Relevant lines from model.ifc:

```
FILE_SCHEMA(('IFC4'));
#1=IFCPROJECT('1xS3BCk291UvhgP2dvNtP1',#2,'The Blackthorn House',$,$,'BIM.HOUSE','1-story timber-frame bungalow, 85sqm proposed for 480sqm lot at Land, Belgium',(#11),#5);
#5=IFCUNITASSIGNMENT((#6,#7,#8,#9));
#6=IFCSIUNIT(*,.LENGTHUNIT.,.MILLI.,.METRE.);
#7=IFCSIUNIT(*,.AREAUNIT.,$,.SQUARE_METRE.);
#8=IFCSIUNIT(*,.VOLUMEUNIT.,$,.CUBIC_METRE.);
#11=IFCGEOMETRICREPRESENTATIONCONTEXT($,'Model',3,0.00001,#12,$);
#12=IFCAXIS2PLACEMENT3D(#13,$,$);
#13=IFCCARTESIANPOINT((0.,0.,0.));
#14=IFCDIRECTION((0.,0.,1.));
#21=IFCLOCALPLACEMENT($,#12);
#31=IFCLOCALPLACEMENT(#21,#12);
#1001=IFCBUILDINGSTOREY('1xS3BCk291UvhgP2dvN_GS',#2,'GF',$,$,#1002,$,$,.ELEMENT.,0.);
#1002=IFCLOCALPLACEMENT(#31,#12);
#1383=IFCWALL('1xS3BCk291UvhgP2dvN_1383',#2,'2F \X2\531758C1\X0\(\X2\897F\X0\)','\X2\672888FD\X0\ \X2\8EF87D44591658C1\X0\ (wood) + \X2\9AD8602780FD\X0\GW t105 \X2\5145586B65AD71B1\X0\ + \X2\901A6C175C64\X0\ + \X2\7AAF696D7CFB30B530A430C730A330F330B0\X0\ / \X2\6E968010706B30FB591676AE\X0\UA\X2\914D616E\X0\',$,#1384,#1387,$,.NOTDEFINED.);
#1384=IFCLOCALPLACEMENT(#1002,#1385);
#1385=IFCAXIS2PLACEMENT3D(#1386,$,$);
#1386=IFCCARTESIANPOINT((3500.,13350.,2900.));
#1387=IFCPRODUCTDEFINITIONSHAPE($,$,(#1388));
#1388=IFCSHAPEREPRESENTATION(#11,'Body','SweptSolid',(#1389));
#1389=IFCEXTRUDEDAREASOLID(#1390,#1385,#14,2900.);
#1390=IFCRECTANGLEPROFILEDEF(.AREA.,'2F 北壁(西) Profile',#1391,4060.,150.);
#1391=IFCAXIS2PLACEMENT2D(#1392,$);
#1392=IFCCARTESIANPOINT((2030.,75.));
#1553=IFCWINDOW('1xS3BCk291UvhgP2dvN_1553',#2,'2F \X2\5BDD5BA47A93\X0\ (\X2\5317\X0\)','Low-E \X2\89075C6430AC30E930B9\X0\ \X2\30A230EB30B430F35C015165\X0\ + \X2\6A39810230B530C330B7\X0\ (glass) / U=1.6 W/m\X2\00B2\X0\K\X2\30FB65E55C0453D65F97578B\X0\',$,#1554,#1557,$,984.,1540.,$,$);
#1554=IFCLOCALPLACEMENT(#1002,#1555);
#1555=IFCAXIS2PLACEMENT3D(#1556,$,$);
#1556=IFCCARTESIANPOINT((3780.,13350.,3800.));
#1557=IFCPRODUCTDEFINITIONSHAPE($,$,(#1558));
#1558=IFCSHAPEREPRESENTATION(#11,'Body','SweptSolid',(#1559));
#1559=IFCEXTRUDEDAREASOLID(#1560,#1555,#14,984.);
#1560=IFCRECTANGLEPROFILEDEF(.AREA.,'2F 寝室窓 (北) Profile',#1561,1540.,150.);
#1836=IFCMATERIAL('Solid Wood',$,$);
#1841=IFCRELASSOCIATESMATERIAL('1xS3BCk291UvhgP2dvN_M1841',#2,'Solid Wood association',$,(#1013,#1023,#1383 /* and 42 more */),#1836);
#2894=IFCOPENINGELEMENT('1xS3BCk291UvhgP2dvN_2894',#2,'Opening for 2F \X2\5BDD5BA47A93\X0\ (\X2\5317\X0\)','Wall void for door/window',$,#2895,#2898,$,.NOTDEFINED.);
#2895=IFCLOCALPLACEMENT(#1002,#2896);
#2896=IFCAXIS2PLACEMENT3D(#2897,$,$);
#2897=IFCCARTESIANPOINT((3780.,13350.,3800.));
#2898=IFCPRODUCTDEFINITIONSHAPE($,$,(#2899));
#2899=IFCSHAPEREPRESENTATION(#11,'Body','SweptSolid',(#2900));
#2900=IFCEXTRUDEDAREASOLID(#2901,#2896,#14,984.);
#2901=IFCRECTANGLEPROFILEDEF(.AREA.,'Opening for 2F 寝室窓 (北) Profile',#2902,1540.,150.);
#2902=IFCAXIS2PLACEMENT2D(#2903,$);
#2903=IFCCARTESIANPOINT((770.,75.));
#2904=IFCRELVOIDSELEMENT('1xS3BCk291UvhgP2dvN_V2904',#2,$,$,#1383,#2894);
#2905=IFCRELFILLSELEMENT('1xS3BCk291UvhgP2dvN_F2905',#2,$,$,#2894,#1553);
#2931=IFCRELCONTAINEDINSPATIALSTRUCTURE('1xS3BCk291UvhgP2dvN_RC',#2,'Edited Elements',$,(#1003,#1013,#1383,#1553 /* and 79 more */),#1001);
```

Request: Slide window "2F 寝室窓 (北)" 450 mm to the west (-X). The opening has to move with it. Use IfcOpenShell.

```python
import ifcopenshell
import ifcopenshell.api.geometry
import ifcopenshell.util.placement

model = ifcopenshell.open("model.ifc")

window = model.by_id(1553)
opening = window.FillsVoids[0].RelatingOpeningElement
wall = opening.VoidsElements[0].RelatingBuildingElement

wall_matrix = ifcopenshell.util.placement.get_local_placement(wall.ObjectPlacement)
shift = wall_matrix[:3, 0] * -450.0
before = ifcopenshell.util.placement.get_local_placement(window.ObjectPlacement)[:3, 3].copy()

# The window is not placed relative to its opening, so move both.
for product in (opening, window):
    matrix = ifcopenshell.util.placement.get_local_placement(product.ObjectPlacement)
    matrix[:3, 3] += shift
    ifcopenshell.api.geometry.edit_object_placement(model, product=product, matrix=matrix, is_si=False)

after = ifcopenshell.util.placement.get_local_placement(window.ObjectPlacement)[:3, 3]
print("window moved by", (after - before).round(3) + 0.0)

model.write("model_edited.ifc")
```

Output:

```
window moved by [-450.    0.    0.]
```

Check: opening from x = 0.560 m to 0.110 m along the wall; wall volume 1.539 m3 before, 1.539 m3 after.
